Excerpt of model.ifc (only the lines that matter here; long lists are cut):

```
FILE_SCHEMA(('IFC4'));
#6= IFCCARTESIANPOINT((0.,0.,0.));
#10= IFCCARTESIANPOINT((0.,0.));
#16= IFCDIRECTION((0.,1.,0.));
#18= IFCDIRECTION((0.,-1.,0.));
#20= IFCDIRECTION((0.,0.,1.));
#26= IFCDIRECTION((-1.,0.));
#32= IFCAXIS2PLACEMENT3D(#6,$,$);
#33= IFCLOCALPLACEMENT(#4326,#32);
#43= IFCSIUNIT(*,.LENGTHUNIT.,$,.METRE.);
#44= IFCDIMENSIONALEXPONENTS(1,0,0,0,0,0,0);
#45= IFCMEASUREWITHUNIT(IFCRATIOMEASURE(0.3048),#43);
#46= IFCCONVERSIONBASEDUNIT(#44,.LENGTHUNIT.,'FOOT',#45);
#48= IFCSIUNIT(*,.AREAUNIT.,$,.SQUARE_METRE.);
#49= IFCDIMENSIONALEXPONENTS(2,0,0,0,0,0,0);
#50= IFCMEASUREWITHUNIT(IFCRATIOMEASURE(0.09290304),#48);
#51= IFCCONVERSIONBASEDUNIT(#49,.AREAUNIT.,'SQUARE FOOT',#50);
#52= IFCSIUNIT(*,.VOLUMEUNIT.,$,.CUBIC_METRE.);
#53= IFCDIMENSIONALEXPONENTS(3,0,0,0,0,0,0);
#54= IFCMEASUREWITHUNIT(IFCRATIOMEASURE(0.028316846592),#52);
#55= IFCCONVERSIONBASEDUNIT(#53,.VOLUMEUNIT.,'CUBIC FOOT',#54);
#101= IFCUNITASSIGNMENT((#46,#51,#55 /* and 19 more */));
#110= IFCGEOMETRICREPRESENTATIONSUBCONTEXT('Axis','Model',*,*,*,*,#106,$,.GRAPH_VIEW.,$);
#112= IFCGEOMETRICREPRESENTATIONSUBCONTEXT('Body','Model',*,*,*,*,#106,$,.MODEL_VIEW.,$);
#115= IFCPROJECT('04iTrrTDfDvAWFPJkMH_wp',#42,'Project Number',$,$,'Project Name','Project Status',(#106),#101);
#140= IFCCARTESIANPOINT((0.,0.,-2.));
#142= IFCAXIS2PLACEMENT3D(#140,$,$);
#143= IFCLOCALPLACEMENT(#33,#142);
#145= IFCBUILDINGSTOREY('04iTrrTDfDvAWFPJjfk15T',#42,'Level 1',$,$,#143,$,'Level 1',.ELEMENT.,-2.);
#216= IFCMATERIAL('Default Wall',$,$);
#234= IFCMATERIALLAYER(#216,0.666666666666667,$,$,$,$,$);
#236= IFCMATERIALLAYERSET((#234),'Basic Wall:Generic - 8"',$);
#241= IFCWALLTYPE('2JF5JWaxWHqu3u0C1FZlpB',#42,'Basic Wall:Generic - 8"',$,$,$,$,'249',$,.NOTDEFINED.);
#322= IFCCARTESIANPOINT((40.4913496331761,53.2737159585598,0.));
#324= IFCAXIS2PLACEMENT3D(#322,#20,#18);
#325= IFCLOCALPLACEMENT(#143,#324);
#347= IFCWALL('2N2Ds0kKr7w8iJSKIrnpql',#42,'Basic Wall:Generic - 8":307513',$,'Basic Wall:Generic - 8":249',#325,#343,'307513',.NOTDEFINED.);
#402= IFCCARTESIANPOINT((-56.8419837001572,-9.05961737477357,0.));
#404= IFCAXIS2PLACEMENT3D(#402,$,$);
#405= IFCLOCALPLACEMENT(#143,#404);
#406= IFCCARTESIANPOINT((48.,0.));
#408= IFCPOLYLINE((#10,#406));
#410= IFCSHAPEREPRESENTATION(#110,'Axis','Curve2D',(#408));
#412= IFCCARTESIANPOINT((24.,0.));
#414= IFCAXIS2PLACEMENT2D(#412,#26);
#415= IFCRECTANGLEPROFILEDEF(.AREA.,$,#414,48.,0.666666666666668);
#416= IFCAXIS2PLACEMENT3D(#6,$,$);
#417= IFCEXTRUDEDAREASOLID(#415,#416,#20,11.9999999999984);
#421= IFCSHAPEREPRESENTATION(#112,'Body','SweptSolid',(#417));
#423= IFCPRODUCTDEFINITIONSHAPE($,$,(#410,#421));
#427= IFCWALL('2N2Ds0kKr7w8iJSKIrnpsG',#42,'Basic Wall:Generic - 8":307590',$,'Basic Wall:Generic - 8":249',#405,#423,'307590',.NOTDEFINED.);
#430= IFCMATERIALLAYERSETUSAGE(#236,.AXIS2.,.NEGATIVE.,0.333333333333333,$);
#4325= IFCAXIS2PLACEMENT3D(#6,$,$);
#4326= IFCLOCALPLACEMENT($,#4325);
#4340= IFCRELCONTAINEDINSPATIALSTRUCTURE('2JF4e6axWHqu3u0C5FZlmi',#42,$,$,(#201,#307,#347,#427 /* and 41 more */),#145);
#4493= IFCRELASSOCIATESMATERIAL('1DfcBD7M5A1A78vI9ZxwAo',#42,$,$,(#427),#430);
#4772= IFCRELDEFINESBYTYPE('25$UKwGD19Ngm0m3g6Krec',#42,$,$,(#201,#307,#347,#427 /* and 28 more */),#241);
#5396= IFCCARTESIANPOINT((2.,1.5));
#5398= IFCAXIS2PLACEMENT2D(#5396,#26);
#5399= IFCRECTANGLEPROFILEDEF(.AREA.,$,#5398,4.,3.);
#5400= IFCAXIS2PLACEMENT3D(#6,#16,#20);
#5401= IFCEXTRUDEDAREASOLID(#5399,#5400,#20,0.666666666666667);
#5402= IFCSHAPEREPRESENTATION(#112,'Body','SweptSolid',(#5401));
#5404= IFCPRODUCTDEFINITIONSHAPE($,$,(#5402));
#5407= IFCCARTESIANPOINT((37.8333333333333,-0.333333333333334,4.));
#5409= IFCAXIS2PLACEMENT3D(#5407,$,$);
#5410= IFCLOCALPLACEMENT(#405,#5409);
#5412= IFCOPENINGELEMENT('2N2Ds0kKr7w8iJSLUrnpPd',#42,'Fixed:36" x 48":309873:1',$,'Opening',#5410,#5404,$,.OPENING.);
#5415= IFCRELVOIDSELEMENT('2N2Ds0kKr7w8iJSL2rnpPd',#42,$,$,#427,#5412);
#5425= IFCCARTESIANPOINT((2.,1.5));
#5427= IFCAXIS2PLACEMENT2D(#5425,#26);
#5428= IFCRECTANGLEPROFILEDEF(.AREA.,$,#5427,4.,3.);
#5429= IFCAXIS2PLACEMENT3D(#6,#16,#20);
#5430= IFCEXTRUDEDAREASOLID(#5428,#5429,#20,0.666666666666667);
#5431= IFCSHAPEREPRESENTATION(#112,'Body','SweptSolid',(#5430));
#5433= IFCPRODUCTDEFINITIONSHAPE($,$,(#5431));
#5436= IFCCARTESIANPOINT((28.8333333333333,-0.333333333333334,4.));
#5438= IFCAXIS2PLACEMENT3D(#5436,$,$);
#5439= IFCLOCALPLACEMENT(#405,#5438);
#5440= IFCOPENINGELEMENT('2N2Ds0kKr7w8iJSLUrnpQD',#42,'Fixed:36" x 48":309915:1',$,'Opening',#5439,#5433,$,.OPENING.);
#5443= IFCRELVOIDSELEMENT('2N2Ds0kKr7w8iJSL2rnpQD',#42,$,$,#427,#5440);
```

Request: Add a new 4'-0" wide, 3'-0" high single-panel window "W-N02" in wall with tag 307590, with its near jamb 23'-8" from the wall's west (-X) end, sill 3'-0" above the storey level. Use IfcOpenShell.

```python
import numpy as np
import ifcopenshell
import ifcopenshell.api.feature
import ifcopenshell.api.geometry
import ifcopenshell.api.root
import ifcopenshell.api.spatial
import ifcopenshell.geom
import ifcopenshell.util.element
import ifcopenshell.util.placement
import ifcopenshell.util.representation
import ifcopenshell.util.shape
import ifcopenshell.util.unit

model = ifcopenshell.open("model.ifc")
unit_scale = ifcopenshell.util.unit.calculate_unit_scale(model)
settings = ifcopenshell.geom.settings()


def volume(element):
    """Net volume in cubic metres, openings subtracted."""
    shape = ifcopenshell.geom.create_shape(settings, element)
    return ifcopenshell.util.shape.get_volume(shape.geometry)


wall = model.by_guid("2N2Ds0kKr7w8iJSKIrnpsG")
storey = ifcopenshell.util.element.get_container(wall, ifc_class="IfcBuildingStorey")
context = ifcopenshell.util.representation.get_context(model, "Model", "Body", "MODEL_VIEW")
before = volume(wall)

width, height, from_end, sill = 1.2192, 0.9144, 7.2136, 0.9144  # metres

# The wall runs along its own X axis, and the end named is its -X end.
wall_shape = ifcopenshell.geom.create_shape(settings, wall)
x, y, z = ifcopenshell.util.shape.get_vertices(wall_shape.geometry).T
start = x.min() + from_end
face, thickness = float(y.min()), float(y.max() - y.min())
wall_matrix = ifcopenshell.util.placement.get_local_placement(wall.ObjectPlacement)
level = ifcopenshell.util.placement.get_local_placement(storey.ObjectPlacement)[2, 3]


def in_wall(x, y):
    """Placement at x, y metres in the wall's axes, at sill height."""
    matrix = wall_matrix.copy()
    matrix[:, 3] = wall_matrix @ np.array([x / unit_scale, y / unit_scale, 0.0, 1.0])
    matrix[2, 3] = level + sill / unit_scale
    return matrix


# Opening: a box that overshoots both wall faces by 50 mm.
opening = ifcopenshell.api.root.create_entity(model, ifc_class="IfcOpeningElement", predefined_type="OPENING")
box = ifcopenshell.api.geometry.add_wall_representation(
    model, context=context, length=width, height=height, thickness=thickness + 0.1
)
ifcopenshell.api.geometry.assign_representation(model, product=opening, representation=box)
ifcopenshell.api.geometry.edit_object_placement(model, product=opening, matrix=in_wall(start, face - 0.05), is_si=False)
ifcopenshell.api.feature.add_feature(model, feature=opening, element=wall)

window = ifcopenshell.api.root.create_entity(model, ifc_class="IfcWindow", name="W-N02", predefined_type="WINDOW")
window.OverallWidth, window.OverallHeight = width / unit_scale, height / unit_scale
window.PartitioningType = "SINGLE_PANEL"
body = ifcopenshell.api.geometry.add_window_representation(
    model,
    context=context,
    overall_width=window.OverallWidth,
    overall_height=window.OverallHeight,
    partition_type="SINGLE_PANEL",
)
ifcopenshell.api.geometry.assign_representation(model, product=window, representation=body)
ifcopenshell.api.spatial.assign_container(model, products=[window], relating_structure=storey)
ifcopenshell.api.feature.add_filling(model, opening=opening, element=window)

# Centre the window in the wall's thickness.
ifcopenshell.api.geometry.edit_object_placement(model, product=window, matrix=in_wall(start, face), is_si=False)
window_shape = ifcopenshell.geom.create_shape(settings, window)
depth = ifcopenshell.util.shape.get_vertices(window_shape.geometry)[:, 1]
offset = face + thickness / 2 - (depth.min() + depth.max()) / 2
ifcopenshell.api.geometry.edit_object_placement(model, product=window, matrix=in_wall(start, offset), is_si=False)

after = volume(wall)

print(f"wall volume {before:.3f} -> {after:.3f} m3")

model.write("model-out.ifc")
```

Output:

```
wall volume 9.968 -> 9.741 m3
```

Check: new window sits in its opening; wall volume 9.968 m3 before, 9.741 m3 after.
